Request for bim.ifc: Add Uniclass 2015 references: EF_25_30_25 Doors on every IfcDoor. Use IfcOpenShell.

First a look at what the model holds.

```python
import ifcopenshell

model = ifcopenshell.open("bim.ifc")
print(model.schema)
print("classifications:", [c.Name for c in model.by_type("IfcClassification")])
for ifc_class in ("IfcDoor", "IfcRoof", "IfcStair", "IfcWall", "IfcWindow"):
    print(ifc_class, len(model.by_type(ifc_class)))
```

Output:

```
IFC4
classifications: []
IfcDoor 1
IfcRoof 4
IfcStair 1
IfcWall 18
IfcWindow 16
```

```python
import ifcopenshell
import ifcopenshell.api.classification

model = ifcopenshell.open("bim.ifc")

system = ifcopenshell.api.classification.add_classification(model, classification="Uniclass 2015")

codes = {
    "IfcDoor": ("EF_25_30_25", "Doors"),
}
for ifc_class, (code, name) in codes.items():
    products = model.by_type(ifc_class)
    ifcopenshell.api.classification.add_reference(
        model, products=products, classification=system, identification=code, name=name
    )
    print(code, len(products))

model.write("bim_rev.ifc")
```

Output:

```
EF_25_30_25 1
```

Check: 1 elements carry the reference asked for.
